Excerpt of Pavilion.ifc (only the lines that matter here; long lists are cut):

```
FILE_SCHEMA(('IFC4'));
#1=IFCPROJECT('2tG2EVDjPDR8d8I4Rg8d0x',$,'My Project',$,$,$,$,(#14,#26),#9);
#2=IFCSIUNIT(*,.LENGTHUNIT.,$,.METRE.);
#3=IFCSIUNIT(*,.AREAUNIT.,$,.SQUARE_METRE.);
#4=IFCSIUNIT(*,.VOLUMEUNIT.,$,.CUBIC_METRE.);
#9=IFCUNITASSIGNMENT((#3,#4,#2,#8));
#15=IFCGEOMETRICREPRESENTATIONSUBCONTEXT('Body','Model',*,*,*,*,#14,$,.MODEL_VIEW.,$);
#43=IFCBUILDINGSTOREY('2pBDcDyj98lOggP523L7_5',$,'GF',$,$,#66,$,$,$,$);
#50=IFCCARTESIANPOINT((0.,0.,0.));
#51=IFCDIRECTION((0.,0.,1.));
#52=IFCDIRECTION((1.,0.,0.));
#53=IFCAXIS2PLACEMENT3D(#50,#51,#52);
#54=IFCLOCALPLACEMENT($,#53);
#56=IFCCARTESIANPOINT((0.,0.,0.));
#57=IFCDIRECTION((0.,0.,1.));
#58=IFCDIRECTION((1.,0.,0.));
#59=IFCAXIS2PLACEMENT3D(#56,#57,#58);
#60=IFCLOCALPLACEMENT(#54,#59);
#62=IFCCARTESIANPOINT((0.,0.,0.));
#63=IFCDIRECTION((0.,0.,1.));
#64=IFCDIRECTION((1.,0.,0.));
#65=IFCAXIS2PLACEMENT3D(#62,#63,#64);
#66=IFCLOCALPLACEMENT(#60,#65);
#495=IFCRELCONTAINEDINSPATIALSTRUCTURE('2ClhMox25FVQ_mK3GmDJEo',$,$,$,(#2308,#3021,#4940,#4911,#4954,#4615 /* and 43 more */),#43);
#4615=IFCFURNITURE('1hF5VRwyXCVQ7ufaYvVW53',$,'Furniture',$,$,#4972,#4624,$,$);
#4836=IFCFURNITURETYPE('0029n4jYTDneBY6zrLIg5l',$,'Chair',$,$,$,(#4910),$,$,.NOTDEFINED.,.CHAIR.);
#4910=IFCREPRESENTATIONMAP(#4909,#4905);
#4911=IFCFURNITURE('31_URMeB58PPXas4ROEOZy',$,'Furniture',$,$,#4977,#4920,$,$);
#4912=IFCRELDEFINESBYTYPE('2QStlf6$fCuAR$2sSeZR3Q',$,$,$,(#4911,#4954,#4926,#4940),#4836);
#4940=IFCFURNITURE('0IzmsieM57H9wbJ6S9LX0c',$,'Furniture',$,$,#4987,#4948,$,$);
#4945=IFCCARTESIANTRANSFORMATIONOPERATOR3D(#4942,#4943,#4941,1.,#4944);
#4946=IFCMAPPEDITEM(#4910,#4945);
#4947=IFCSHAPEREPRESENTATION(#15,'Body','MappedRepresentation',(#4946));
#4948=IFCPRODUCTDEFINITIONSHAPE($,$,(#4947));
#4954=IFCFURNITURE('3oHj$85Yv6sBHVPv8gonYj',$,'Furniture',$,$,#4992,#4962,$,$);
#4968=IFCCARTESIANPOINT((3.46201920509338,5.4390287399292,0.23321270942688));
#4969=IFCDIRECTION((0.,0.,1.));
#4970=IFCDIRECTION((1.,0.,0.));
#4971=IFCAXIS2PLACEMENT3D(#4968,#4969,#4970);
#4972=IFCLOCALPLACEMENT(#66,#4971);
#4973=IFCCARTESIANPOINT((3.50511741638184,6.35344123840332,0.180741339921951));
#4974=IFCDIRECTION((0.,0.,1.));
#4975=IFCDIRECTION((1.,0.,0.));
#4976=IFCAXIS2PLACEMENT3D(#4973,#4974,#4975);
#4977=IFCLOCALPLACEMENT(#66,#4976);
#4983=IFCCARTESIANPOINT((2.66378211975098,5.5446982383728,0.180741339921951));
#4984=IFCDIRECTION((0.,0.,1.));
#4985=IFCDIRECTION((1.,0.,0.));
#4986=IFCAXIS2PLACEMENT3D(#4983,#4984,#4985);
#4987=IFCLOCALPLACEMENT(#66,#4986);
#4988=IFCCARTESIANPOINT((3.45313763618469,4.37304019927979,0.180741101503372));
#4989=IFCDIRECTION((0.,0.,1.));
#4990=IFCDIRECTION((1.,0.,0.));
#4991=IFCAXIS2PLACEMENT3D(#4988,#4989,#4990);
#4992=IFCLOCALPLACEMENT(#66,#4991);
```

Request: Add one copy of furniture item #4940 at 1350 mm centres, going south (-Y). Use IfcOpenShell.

```python
import numpy as np
import ifcopenshell
import ifcopenshell.api.geometry
import ifcopenshell.api.root
import ifcopenshell.util.element
import ifcopenshell.util.placement

model = ifcopenshell.open("Pavilion.ifc")

source = model.by_guid("0IzmsieM57H9wbJ6S9LX0c")
base = ifcopenshell.util.placement.get_local_placement(source.ObjectPlacement)
step = np.array([0.0, -1.0, 0.0]) * 1.35

for i in range(1, 2):
    copy = ifcopenshell.api.root.copy_class(model, product=source)
    copy.Representation = ifcopenshell.util.element.copy_deep(
        model, source.Representation, exclude=["IfcGeometricRepresentationContext", "IfcRepresentationMap"]
    )
    matrix = base.copy()
    matrix[:3, 3] += i * step
    print("added at", matrix[:3, 3].round(3) + 0.0)
    ifcopenshell.api.geometry.edit_object_placement(model, product=copy, matrix=matrix, is_si=False)

model.write("Pavilion_updated.ifc")
```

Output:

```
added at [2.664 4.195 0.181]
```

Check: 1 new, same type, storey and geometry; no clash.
